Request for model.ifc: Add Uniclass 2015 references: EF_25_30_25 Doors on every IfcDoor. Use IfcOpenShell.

First a look at what the model holds.

```python
import ifcopenshell

model = ifcopenshell.open("model.ifc")
print(model.schema)
print("classifications:", [c.Name for c in model.by_type("IfcClassification")])
for ifc_class in ("IfcDoor", "IfcRoof", "IfcStair", "IfcWall", "IfcWindow"):
    print(ifc_class, len(model.by_type(ifc_class)))
```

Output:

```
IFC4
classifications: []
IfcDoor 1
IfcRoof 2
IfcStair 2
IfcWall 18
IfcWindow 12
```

```python
import ifcopenshell
import ifcopenshell.api.classification

model = ifcopenshell.open("model.ifc")

system = ifcopenshell.api.classification.add_classification(model, classification="Uniclass 2015")

codes = {
    "IfcDoor": ("EF_25_30_25", "Doors"),
}
for ifc_class, (code, name) in codes.items():
    products = model.by_type(ifc_class)
    ifcopenshell.api.classification.add_reference(
        model, products=products, classification=system, identification=code, name=name
    )
    print(code, len(products))

model.write("model_v2.ifc")
```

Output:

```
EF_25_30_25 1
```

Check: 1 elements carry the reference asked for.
